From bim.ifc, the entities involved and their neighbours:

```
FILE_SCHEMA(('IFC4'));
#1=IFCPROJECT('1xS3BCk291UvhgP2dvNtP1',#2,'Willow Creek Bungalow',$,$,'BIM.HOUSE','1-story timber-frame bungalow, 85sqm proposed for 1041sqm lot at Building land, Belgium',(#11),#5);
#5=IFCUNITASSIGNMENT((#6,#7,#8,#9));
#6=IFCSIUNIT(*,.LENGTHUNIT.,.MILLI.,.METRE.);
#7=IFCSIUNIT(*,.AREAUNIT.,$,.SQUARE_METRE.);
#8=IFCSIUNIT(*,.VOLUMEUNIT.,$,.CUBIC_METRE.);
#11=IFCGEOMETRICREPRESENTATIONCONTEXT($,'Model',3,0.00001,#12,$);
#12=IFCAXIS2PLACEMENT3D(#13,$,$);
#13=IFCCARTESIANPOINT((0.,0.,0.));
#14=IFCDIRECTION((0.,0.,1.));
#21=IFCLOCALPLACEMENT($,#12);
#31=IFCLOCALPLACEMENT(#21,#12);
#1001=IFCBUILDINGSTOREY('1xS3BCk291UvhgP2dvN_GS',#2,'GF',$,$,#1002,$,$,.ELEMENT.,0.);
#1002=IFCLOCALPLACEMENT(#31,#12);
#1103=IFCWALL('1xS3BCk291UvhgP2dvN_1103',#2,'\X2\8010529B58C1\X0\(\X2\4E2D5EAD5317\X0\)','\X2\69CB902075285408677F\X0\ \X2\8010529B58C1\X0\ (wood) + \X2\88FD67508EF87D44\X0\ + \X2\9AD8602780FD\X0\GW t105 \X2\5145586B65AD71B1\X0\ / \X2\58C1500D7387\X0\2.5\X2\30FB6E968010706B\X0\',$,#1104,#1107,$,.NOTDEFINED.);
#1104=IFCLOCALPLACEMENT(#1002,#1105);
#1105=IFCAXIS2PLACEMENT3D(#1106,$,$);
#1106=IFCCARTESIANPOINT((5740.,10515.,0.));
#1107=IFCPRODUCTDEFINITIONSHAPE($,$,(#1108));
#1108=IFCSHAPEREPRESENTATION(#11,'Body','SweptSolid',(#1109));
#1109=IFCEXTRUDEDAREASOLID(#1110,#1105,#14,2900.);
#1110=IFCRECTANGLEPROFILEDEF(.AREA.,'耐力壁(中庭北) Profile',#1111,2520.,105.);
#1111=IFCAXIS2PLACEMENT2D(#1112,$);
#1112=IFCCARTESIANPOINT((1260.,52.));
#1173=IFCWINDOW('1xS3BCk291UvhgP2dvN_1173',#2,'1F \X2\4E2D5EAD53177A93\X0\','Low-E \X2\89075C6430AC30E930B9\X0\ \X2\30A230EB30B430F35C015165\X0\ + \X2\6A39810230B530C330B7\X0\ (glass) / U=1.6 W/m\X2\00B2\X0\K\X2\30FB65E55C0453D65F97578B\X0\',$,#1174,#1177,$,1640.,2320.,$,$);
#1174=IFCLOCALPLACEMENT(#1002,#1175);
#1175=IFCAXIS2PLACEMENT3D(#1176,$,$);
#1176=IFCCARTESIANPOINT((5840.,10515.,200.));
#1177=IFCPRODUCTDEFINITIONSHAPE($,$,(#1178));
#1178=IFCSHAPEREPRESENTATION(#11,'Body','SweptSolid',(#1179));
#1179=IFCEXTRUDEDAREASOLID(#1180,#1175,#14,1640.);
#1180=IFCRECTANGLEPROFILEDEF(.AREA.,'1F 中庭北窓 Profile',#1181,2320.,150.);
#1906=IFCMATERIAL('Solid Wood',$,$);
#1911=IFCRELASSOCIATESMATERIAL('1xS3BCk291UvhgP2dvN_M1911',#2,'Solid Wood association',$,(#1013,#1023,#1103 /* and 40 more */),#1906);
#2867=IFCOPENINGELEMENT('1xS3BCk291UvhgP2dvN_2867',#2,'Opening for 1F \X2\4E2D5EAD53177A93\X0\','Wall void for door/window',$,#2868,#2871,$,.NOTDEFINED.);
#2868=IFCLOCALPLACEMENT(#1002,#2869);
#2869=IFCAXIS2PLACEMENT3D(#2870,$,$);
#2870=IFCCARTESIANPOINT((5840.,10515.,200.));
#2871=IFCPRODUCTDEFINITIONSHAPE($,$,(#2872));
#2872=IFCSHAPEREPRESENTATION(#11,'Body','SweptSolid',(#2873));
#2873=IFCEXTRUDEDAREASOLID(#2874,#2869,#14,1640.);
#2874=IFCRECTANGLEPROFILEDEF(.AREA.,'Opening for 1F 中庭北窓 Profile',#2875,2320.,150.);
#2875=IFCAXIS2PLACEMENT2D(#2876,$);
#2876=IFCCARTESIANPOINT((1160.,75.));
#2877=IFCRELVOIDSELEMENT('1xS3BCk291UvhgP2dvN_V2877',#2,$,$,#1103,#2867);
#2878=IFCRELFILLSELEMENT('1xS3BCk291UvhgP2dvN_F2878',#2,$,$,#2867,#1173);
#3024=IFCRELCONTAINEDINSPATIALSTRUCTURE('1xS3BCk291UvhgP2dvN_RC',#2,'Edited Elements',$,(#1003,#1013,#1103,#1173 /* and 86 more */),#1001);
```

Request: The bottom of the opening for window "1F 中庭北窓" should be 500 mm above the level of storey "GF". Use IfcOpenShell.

```python
import numpy as np
import ifcopenshell
import ifcopenshell.api.geometry
import ifcopenshell.geom
import ifcopenshell.util.element
import ifcopenshell.util.placement
import ifcopenshell.util.shape
import ifcopenshell.util.unit

model = ifcopenshell.open("bim.ifc")
unit_scale = ifcopenshell.util.unit.calculate_unit_scale(model)

window = model.by_id(1173)
opening = window.FillsVoids[0].RelatingOpeningElement
storey = ifcopenshell.util.element.get_container(window, ifc_class="IfcBuildingStorey")
level = ifcopenshell.util.placement.get_local_placement(storey.ObjectPlacement)[2, 3]

# The opening's origin need not be at the sill, so measure its lowest point.
shape = ifcopenshell.geom.create_shape(ifcopenshell.geom.settings(), opening)
bottom = ifcopenshell.util.shape.get_shape_bottom_elevation(shape, shape.geometry) / unit_scale
dz = level + 0.5 / unit_scale - bottom

shift = np.array([0.0, 0.0, dz])
# The window is not placed relative to its opening, so move both.
for product in (opening, window):
    matrix = ifcopenshell.util.placement.get_local_placement(product.ObjectPlacement)
    matrix[:3, 3] += shift
    ifcopenshell.api.geometry.edit_object_placement(model, product=product, matrix=matrix, is_si=False)

print(f"moved by {dz * unit_scale:+.3f} m")

model.write("bim-out.ifc")
```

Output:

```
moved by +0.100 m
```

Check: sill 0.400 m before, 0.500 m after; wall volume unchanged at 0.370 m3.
